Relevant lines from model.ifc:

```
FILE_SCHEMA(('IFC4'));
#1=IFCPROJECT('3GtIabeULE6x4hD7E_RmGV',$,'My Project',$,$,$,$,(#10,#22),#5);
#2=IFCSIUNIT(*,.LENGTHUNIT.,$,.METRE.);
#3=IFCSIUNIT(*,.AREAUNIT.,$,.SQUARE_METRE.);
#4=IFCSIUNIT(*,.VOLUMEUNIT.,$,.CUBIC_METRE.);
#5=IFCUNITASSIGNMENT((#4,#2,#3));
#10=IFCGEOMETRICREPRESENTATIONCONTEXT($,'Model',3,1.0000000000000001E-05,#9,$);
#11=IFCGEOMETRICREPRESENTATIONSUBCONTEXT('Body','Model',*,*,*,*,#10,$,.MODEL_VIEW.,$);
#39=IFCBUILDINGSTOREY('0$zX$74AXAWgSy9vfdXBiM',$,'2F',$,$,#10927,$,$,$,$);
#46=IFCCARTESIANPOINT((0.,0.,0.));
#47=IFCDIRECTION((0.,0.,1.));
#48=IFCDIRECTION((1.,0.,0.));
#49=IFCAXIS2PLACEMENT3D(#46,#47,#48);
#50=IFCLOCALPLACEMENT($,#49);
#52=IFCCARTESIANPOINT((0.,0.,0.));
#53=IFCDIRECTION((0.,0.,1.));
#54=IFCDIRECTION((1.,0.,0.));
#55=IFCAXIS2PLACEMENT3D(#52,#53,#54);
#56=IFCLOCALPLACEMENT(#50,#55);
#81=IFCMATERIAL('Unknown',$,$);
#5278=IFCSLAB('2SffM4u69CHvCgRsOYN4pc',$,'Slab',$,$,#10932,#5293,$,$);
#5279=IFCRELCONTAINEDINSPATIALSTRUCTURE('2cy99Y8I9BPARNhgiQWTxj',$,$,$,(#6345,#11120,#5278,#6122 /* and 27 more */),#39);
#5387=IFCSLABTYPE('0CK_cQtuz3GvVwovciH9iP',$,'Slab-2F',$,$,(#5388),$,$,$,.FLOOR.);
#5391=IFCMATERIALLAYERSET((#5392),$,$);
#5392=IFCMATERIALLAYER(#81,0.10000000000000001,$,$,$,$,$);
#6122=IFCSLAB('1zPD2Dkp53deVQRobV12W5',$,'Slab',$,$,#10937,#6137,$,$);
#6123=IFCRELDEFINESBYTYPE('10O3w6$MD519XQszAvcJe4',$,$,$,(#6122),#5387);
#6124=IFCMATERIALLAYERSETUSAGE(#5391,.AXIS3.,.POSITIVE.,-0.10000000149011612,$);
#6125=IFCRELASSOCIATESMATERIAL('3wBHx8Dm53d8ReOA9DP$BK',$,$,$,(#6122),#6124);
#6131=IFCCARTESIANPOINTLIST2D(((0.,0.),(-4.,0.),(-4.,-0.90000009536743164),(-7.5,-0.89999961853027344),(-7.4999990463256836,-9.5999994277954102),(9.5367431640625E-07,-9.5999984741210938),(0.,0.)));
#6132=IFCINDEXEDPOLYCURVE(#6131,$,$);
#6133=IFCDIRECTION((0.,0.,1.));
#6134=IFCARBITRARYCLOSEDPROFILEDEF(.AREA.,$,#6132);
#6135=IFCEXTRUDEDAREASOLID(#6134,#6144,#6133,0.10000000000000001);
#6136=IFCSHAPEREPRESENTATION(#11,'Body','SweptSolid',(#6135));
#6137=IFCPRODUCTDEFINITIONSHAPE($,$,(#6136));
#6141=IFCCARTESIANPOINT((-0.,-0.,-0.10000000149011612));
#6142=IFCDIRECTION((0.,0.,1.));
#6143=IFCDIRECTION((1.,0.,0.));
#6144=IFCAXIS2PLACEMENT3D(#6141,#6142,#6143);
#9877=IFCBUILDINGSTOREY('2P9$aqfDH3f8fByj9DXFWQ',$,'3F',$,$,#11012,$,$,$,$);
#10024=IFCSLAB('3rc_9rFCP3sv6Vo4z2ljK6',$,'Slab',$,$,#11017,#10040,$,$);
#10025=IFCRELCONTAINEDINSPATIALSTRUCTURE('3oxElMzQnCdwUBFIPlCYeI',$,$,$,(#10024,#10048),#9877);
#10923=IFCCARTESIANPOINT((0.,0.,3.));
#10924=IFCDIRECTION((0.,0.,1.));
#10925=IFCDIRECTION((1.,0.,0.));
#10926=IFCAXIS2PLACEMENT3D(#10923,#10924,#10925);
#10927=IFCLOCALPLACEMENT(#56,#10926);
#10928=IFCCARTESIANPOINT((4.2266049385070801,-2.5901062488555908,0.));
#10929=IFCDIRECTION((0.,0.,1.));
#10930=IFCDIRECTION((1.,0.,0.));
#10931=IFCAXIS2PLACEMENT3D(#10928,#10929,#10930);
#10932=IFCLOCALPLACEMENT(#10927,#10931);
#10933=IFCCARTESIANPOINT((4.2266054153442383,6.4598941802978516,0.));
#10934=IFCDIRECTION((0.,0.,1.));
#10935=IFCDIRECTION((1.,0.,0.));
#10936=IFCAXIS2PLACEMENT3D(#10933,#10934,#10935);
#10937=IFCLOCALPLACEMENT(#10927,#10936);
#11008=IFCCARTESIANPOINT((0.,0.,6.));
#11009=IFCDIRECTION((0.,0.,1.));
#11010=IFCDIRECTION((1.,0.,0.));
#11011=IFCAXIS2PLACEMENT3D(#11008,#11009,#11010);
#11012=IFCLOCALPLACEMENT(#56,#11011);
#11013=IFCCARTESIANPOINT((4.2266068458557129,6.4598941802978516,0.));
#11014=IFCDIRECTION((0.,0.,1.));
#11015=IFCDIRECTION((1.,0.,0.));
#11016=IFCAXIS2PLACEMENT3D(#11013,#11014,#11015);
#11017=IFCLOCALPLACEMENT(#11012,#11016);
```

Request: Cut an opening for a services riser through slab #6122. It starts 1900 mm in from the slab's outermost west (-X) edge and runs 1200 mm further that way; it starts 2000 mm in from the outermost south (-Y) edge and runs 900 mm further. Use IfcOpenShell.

```python
import numpy as np
import ifcopenshell
import ifcopenshell.api.feature
import ifcopenshell.api.geometry
import ifcopenshell.api.root
import ifcopenshell.geom
import ifcopenshell.util.placement
import ifcopenshell.util.representation
import ifcopenshell.util.shape
import ifcopenshell.util.unit

model = ifcopenshell.open("model.ifc")
unit_scale = ifcopenshell.util.unit.calculate_unit_scale(model)
settings = ifcopenshell.geom.settings()


def volume(element):
    """Net volume in cubic metres, openings subtracted."""
    shape = ifcopenshell.geom.create_shape(settings, element)
    return ifcopenshell.util.shape.get_volume(shape.geometry)


slab = model.by_guid("1zPD2Dkp53deVQRobV12W5")
before = volume(slab)

# Extent in the slab's own axes, in metres. The edges named are its -X and -Y sides.
slab_shape = ifcopenshell.geom.create_shape(settings, slab)
vertices = ifcopenshell.util.shape.get_vertices(slab_shape.geometry)
x_min, y_min, bottom = vertices.min(axis=0)
top = vertices[:, 2].max()

opening = ifcopenshell.api.root.create_entity(model, ifc_class="IfcOpeningElement", name="Services riser opening", predefined_type="OPENING")
context = ifcopenshell.util.representation.get_context(model, "Model", "Body", "MODEL_VIEW")
width, depth = 1.2, 0.9
outline = [(0.0, 0.0), (width, 0.0), (width, depth), (0.0, depth), (0.0, 0.0)]
# Overshoot both faces by 50 mm so the cut is clean.
shape = ifcopenshell.api.geometry.add_slab_representation(
    model, context=context, depth=top - bottom + 0.1, polyline=outline
)
ifcopenshell.api.geometry.assign_representation(model, product=opening, representation=shape)

matrix = ifcopenshell.util.placement.get_local_placement(slab.ObjectPlacement)
matrix[:, 3] = matrix @ np.append(np.array([x_min + 1.9, y_min + 2, bottom - 0.05]) / unit_scale, 1.0)
ifcopenshell.api.geometry.edit_object_placement(model, product=opening, matrix=matrix, is_si=False)
ifcopenshell.api.feature.add_feature(model, feature=opening, element=slab)

after = volume(slab)

print(f"slab volume {before:.3f} -> {after:.3f} m3")

model.write("model_rev.ifc")
```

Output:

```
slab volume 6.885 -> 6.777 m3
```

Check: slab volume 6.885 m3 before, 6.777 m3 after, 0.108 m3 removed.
